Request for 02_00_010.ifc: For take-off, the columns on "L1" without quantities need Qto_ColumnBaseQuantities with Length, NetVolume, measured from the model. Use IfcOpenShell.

First a look at what the model holds.

```python
import ifcopenshell
import ifcopenshell.util.element
import ifcopenshell.util.unit

model = ifcopenshell.open("02_00_010.ifc")
print(model.schema)
for unit_type in ("LENGTHUNIT", "AREAUNIT", "VOLUMEUNIT"):
    print(unit_type, ifcopenshell.util.unit.calculate_unit_scale(model, unit_type))
storey = next(s for s in model.by_type("IfcBuildingStorey") if s.Name == "L1")
columns = [e for e in ifcopenshell.util.element.get_decomposition(storey) if e.is_a("IfcColumn")]
for e in sorted(columns, key=lambda e: e.id()):
    print(e.id(), e.is_a(), e.Name, list(ifcopenshell.util.element.get_psets(e, qtos_only=True)), sep=" | ")
```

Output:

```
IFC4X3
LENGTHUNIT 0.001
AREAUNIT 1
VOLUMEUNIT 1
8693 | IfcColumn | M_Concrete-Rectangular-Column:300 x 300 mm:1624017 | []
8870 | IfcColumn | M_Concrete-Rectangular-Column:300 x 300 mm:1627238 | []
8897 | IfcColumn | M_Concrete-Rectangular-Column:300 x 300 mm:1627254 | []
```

```python
import ifcopenshell
import ifcopenshell.api.pset
import ifcopenshell.geom
import ifcopenshell.util.element
import ifcopenshell.util.shape
import ifcopenshell.util.unit

model = ifcopenshell.open("02_00_010.ifc")
unit_scale = ifcopenshell.util.unit.calculate_unit_scale(model)
volume_scale = ifcopenshell.util.unit.calculate_unit_scale(model, "VOLUMEUNIT")
settings = ifcopenshell.geom.settings()

storey = next(s for s in model.by_type("IfcBuildingStorey") if s.Name == "L1")
columns = [e for e in ifcopenshell.util.element.get_decomposition(storey) if e.is_a("IfcColumn")]

for e in sorted(columns, key=lambda e: e.id()):
    if ifcopenshell.util.element.get_psets(e, qtos_only=True, should_inherit=False):
        continue
    # Geometry comes back in metres, in the element's own axes.
    shape = ifcopenshell.geom.create_shape(settings, e)
    values = {
        "Length": ifcopenshell.util.shape.get_z(shape.geometry) / unit_scale,
        "NetVolume": ifcopenshell.util.shape.get_volume(shape.geometry) / volume_scale,
    }
    qto = ifcopenshell.api.pset.add_qto(model, product=e, name="Qto_ColumnBaseQuantities")
    ifcopenshell.api.pset.edit_qto(model, qto=qto, properties=values)
    print(e.id(), {k: round(v, 3) for k, v in values.items()})

model.write("02_00_010_v2.ifc")
```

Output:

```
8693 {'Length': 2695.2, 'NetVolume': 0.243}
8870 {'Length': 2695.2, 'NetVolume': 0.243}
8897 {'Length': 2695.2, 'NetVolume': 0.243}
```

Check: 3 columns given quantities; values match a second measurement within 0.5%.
